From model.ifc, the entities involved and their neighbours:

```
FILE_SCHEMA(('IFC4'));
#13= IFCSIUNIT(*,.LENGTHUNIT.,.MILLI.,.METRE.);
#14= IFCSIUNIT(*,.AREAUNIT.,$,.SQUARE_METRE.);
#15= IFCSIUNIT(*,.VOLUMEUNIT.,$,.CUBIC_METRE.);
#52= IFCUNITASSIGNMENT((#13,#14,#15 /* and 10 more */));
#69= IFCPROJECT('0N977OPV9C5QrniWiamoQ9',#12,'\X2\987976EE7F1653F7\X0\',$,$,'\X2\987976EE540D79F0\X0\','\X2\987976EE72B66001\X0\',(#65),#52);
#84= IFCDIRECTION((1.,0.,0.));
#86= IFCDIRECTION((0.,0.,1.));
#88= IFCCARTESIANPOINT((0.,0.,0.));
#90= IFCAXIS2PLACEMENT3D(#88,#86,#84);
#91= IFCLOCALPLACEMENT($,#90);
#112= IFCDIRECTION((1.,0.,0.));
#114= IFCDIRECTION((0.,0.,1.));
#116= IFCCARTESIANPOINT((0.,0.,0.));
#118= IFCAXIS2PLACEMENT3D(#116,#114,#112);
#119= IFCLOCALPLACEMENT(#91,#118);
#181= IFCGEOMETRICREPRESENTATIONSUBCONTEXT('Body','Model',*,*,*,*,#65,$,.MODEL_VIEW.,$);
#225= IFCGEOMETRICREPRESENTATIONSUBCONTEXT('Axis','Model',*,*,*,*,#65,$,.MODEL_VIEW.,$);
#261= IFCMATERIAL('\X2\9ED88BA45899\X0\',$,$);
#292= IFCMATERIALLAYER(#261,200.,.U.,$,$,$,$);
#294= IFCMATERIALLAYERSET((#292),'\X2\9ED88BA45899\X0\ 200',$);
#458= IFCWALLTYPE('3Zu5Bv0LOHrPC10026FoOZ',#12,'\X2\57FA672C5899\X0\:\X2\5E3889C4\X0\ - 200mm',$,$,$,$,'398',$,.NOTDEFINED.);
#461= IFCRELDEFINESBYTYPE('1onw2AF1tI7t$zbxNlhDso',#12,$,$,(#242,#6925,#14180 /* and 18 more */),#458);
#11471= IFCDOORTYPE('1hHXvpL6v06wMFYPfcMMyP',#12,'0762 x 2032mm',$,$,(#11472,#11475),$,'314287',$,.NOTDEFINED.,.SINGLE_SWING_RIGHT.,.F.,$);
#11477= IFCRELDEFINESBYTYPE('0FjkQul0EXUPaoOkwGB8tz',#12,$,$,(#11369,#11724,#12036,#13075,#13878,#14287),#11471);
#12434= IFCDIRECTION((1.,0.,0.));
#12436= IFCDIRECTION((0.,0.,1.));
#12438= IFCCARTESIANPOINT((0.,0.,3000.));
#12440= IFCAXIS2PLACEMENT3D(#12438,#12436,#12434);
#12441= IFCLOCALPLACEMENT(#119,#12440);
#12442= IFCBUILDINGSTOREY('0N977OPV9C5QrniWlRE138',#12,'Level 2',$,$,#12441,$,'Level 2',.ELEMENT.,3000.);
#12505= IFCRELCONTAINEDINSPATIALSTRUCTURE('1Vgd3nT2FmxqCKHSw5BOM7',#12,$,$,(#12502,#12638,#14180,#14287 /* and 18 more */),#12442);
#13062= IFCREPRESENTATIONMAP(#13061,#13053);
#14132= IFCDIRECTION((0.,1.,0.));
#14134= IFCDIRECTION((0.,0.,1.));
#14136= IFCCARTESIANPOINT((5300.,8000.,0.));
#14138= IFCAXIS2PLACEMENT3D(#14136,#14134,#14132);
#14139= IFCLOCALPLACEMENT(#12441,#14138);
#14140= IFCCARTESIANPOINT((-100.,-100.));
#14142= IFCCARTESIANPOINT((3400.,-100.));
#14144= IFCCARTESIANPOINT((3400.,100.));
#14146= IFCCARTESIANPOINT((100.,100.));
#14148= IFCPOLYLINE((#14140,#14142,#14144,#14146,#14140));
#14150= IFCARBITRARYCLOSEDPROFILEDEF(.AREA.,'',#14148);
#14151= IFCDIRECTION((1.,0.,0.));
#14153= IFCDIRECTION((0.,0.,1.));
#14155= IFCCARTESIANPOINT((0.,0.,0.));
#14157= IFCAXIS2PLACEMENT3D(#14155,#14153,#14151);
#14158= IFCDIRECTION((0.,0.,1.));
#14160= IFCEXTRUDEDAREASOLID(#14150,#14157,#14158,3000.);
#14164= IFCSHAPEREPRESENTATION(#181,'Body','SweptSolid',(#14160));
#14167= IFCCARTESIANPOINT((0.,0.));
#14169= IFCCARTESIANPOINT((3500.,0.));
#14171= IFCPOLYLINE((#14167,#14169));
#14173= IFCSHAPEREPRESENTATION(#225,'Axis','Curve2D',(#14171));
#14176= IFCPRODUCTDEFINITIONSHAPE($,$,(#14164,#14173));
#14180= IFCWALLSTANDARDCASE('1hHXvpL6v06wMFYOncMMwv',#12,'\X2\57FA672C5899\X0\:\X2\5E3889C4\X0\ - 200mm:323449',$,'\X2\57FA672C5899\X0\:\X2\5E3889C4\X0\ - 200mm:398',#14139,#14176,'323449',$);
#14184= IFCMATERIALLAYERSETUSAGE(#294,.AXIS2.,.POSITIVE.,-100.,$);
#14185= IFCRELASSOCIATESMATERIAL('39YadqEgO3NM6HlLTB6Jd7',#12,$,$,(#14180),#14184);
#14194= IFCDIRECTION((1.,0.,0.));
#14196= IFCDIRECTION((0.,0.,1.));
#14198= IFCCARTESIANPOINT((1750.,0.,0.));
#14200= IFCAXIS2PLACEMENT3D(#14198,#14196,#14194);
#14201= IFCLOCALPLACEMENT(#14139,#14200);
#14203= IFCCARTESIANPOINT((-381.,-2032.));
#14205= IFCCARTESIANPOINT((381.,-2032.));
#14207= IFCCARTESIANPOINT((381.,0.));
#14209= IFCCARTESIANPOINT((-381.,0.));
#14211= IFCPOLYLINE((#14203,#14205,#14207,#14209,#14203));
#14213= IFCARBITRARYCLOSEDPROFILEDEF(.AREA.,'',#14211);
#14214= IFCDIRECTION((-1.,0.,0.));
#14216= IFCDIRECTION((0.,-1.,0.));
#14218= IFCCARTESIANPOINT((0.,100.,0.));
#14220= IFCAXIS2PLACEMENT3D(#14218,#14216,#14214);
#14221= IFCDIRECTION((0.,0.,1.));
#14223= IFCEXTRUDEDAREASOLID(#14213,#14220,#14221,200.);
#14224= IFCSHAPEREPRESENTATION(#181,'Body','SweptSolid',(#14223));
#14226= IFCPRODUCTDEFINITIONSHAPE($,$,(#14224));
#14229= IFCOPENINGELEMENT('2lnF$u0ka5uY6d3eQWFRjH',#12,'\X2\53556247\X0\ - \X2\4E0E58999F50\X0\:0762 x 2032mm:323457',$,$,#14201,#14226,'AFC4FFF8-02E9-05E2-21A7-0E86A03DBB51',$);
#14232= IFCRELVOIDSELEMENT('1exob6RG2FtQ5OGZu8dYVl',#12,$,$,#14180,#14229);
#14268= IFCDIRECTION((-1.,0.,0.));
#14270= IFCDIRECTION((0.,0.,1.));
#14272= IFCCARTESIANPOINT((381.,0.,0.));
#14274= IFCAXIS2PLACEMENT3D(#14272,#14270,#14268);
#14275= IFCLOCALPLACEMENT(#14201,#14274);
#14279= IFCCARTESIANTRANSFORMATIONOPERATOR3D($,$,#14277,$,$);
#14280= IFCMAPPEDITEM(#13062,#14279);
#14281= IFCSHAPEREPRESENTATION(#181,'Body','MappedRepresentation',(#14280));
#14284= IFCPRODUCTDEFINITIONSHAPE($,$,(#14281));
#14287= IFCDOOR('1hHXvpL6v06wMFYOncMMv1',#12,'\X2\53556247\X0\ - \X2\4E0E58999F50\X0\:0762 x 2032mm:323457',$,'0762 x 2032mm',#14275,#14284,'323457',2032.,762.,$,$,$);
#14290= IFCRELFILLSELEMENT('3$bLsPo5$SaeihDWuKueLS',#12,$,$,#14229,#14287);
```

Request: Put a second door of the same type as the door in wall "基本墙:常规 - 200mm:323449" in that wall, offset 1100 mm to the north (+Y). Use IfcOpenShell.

```python
import ifcopenshell
import ifcopenshell.api.feature
import ifcopenshell.api.geometry
import ifcopenshell.api.root
import ifcopenshell.geom
import ifcopenshell.util.element
import ifcopenshell.util.placement
import ifcopenshell.util.shape

model = ifcopenshell.open("model.ifc")
settings = ifcopenshell.geom.settings()


def volume(element):
    """Net volume in cubic metres, openings subtracted."""
    shape = ifcopenshell.geom.create_shape(settings, element)
    return ifcopenshell.util.shape.get_volume(shape.geometry)


def reuse_history(source, copy):
    """copy_class also copies each property set's owner history, people and application; keep the originals."""
    for rel in copy.IsDefinedBy:
        if rel.is_a("IfcRelDefinesByProperties") and (history := rel.RelatingPropertyDefinition.OwnerHistory):
            rel.RelatingPropertyDefinition.OwnerHistory = source.OwnerHistory
            ifcopenshell.util.element.remove_deep2(model, history)


door = model.by_guid("1hHXvpL6v06wMFYOncMMv1")
opening = door.FillsVoids[0].RelatingOpeningElement
wall = opening.VoidsElements[0].RelatingBuildingElement
before = volume(wall)
shift = ifcopenshell.util.placement.get_local_placement(wall.ObjectPlacement)[:3, 0] * 1100.0

# copy_class copies the void relationship, type, container and properties, but no geometry.
new_opening = ifcopenshell.api.root.copy_class(model, product=opening)
new_opening.Representation = ifcopenshell.util.element.copy_deep(
    model, opening.Representation, exclude=["IfcGeometricRepresentationContext", "IfcRepresentationMap"]
)
new_opening.Name = "单扇 - 与墙齐:0762 x 2032mm"
new_opening.Tag = None
new_door = ifcopenshell.api.root.copy_class(model, product=door)
new_door.Representation = ifcopenshell.util.element.copy_deep(
    model, door.Representation, exclude=["IfcGeometricRepresentationContext", "IfcRepresentationMap"]
)
new_door.Name = "单扇 - 与墙齐:0762 x 2032mm"
new_door.Tag = None
reuse_history(door, new_door)
ifcopenshell.api.feature.add_filling(model, opening=new_opening, element=new_door)

for old, new in ((opening, new_opening), (door, new_door)):
    matrix = ifcopenshell.util.placement.get_local_placement(old.ObjectPlacement)
    matrix[:3, 3] += shift
    ifcopenshell.api.geometry.edit_object_placement(model, product=new, matrix=matrix, is_si=False)

after = volume(wall)

print(f"wall volume {before:.3f} -> {after:.3f} m3")

model.write("model_updated.ifc")
```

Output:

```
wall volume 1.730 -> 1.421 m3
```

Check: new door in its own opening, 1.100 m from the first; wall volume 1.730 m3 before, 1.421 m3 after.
